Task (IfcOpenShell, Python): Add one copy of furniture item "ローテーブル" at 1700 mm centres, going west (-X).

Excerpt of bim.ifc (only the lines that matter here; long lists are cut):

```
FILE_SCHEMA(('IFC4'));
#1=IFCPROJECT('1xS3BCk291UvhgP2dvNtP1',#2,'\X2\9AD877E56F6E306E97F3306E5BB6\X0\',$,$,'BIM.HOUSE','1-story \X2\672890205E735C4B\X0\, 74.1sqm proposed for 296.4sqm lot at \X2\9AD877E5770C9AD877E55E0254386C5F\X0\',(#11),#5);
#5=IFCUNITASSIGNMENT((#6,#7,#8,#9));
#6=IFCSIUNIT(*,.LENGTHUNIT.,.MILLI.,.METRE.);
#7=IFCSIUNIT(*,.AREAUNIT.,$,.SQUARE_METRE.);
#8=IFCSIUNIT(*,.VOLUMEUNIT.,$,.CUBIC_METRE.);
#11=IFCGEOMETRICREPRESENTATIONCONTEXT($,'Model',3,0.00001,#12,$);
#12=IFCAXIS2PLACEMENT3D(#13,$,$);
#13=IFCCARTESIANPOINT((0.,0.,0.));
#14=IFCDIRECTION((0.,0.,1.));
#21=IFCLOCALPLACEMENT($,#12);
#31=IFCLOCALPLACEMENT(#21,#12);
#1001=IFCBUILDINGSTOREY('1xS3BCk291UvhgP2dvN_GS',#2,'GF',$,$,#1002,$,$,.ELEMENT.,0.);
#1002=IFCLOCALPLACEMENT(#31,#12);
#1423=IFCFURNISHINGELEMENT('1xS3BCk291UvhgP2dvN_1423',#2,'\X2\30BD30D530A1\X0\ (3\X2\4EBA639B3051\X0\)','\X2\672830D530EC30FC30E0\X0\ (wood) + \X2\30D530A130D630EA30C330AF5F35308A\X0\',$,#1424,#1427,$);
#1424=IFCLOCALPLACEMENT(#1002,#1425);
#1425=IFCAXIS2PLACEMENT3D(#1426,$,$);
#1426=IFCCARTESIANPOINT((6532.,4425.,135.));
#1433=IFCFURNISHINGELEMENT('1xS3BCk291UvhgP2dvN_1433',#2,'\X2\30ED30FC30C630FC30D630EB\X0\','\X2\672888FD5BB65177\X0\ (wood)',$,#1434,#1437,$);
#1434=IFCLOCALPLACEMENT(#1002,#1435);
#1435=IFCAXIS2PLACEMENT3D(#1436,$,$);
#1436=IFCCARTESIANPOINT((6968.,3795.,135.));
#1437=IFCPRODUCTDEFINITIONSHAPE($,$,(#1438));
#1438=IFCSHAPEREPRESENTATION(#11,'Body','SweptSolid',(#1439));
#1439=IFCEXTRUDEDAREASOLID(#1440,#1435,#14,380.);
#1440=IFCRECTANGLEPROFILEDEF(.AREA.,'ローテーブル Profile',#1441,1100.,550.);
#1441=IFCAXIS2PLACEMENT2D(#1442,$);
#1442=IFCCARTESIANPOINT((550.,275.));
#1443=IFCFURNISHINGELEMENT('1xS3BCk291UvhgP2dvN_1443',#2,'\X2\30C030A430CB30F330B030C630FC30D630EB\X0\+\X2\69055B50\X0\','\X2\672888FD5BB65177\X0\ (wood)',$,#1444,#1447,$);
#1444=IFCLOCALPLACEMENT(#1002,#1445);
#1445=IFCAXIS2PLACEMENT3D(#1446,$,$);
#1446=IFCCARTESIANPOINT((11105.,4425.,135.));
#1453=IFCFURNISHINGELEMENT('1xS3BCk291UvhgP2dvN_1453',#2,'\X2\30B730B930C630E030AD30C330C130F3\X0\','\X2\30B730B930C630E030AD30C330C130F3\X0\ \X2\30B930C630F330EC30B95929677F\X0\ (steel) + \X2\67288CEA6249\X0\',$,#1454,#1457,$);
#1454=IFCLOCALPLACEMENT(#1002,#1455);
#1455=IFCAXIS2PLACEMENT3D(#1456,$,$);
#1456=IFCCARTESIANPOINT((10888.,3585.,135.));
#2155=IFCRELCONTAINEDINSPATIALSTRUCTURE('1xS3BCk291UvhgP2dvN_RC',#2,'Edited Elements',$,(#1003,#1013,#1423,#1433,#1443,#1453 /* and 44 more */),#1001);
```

```python
import numpy as np
import ifcopenshell
import ifcopenshell.api.geometry
import ifcopenshell.api.root
import ifcopenshell.util.element
import ifcopenshell.util.placement

model = ifcopenshell.open("bim.ifc")


def reuse_history(source, copy):
    """copy_class also copies each property set's owner history, people and application; keep the originals."""
    for rel in copy.IsDefinedBy:
        if rel.is_a("IfcRelDefinesByProperties") and (history := rel.RelatingPropertyDefinition.OwnerHistory):
            rel.RelatingPropertyDefinition.OwnerHistory = source.OwnerHistory
            ifcopenshell.util.element.remove_deep2(model, history)


source = model.by_guid("1xS3BCk291UvhgP2dvN_1433")
base = ifcopenshell.util.placement.get_local_placement(source.ObjectPlacement)
step = np.array([-1.0, 0.0, 0.0]) * 1700.0

for i in range(1, 2):
    copy = ifcopenshell.api.root.copy_class(model, product=source)
    copy.Representation = ifcopenshell.util.element.copy_deep(
        model, source.Representation, exclude=["IfcGeometricRepresentationContext", "IfcRepresentationMap"]
    )
    reuse_history(source, copy)
    matrix = base.copy()
    matrix[:3, 3] += i * step
    print("added at", matrix[:3, 3].round(3) + 0.0)
    ifcopenshell.api.geometry.edit_object_placement(model, product=copy, matrix=matrix, is_si=False)

model.write("bim-out.ifc")
```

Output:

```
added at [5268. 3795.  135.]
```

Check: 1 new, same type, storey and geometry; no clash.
